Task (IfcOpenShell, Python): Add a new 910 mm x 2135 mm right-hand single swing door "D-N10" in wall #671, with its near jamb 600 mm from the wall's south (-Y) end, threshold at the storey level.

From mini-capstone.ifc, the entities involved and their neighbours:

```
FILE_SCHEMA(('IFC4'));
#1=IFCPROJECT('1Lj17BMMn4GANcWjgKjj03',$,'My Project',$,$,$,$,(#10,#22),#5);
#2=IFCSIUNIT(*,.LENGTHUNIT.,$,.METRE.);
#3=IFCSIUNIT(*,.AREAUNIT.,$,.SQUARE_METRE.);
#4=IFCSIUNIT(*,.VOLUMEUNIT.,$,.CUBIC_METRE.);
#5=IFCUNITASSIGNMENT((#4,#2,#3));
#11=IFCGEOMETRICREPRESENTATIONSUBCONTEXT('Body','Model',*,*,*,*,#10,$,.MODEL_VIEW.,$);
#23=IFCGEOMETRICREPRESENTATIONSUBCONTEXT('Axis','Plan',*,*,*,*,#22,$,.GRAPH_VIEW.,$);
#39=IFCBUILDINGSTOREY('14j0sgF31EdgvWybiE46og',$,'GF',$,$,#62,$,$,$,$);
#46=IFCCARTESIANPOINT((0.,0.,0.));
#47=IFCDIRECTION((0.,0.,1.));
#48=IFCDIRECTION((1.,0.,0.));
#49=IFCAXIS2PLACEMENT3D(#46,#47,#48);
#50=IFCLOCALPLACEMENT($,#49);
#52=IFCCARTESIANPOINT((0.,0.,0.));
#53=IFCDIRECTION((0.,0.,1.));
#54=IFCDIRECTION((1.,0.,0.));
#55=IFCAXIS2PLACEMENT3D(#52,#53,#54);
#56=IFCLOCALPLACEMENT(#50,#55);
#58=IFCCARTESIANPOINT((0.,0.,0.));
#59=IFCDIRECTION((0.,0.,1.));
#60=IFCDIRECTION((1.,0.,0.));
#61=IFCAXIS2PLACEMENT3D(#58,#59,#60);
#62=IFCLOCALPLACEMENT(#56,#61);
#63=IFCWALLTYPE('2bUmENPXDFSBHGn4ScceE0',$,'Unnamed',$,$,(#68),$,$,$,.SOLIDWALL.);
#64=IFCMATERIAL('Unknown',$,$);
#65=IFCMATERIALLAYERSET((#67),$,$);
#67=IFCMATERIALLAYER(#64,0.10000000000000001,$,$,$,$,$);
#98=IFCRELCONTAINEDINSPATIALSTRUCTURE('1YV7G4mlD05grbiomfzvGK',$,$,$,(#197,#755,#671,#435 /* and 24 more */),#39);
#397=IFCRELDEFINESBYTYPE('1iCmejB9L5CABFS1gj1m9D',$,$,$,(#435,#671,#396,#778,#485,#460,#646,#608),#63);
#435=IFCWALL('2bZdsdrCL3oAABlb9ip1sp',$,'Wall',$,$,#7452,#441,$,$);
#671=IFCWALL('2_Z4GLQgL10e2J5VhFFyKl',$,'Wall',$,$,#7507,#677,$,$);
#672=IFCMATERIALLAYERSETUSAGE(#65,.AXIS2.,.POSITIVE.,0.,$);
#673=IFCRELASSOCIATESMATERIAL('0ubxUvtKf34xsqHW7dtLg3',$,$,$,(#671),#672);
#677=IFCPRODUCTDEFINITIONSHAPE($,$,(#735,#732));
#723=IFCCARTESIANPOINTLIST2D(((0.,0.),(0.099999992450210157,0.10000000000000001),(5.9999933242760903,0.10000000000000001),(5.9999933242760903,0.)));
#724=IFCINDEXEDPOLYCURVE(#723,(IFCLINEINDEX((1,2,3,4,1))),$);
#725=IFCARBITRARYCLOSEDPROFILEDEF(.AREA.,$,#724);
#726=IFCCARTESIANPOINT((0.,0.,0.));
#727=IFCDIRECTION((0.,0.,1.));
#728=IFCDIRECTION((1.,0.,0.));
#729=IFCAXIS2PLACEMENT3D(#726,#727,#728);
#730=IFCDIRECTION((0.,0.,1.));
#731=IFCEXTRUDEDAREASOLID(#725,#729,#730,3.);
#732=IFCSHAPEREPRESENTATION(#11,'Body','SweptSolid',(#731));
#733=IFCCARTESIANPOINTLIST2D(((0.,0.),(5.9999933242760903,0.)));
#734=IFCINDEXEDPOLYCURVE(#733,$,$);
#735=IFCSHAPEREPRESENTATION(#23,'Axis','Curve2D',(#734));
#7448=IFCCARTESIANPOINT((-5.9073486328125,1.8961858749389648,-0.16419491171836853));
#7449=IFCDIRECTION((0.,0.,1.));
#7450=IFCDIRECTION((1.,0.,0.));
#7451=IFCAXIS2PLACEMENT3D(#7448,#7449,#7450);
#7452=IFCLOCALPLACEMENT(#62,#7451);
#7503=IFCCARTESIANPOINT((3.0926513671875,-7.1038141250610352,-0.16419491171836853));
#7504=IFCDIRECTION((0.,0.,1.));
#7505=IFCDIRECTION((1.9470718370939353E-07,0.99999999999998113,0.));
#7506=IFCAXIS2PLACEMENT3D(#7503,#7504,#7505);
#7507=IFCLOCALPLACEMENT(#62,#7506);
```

```python
import numpy as np
import ifcopenshell
import ifcopenshell.api.feature
import ifcopenshell.api.geometry
import ifcopenshell.api.root
import ifcopenshell.api.spatial
import ifcopenshell.geom
import ifcopenshell.util.element
import ifcopenshell.util.placement
import ifcopenshell.util.representation
import ifcopenshell.util.shape
import ifcopenshell.util.unit

model = ifcopenshell.open("mini-capstone.ifc")
unit_scale = ifcopenshell.util.unit.calculate_unit_scale(model)
settings = ifcopenshell.geom.settings()


def volume(element):
    """Net volume in cubic metres, openings subtracted."""
    shape = ifcopenshell.geom.create_shape(settings, element)
    return ifcopenshell.util.shape.get_volume(shape.geometry)


wall = model.by_guid("2_Z4GLQgL10e2J5VhFFyKl")
storey = ifcopenshell.util.element.get_container(wall, ifc_class="IfcBuildingStorey")
context = ifcopenshell.util.representation.get_context(model, "Model", "Body", "MODEL_VIEW")
before = volume(wall)

width, height, from_end, sill = 0.91, 2.135, 0.6, 0.0  # metres

# The wall runs along its own X axis, and the end named is its -X end.
wall_shape = ifcopenshell.geom.create_shape(settings, wall)
x, y, z = ifcopenshell.util.shape.get_vertices(wall_shape.geometry).T
start = x.min() + from_end
face, thickness = float(y.min()), float(y.max() - y.min())
wall_matrix = ifcopenshell.util.placement.get_local_placement(wall.ObjectPlacement)
level = ifcopenshell.util.placement.get_local_placement(storey.ObjectPlacement)[2, 3]


def in_wall(x, y):
    """Placement at x, y metres in the wall's axes, at sill height."""
    matrix = wall_matrix.copy()
    matrix[:, 3] = wall_matrix @ np.array([x / unit_scale, y / unit_scale, 0.0, 1.0])
    matrix[2, 3] = level + sill / unit_scale
    return matrix


# Opening: a box that overshoots both wall faces by 50 mm.
opening = ifcopenshell.api.root.create_entity(model, ifc_class="IfcOpeningElement", predefined_type="OPENING")
box = ifcopenshell.api.geometry.add_wall_representation(
    model, context=context, length=width, height=height, thickness=thickness + 0.1
)
ifcopenshell.api.geometry.assign_representation(model, product=opening, representation=box)
ifcopenshell.api.geometry.edit_object_placement(model, product=opening, matrix=in_wall(start, face - 0.05), is_si=False)
ifcopenshell.api.feature.add_feature(model, feature=opening, element=wall)

door = ifcopenshell.api.root.create_entity(model, ifc_class="IfcDoor", name="D-N10", predefined_type="DOOR")
door.OverallWidth, door.OverallHeight = width / unit_scale, height / unit_scale
door.OperationType = "SINGLE_SWING_RIGHT"
body = ifcopenshell.api.geometry.add_door_representation(
    model,
    context=context,
    overall_width=door.OverallWidth,
    overall_height=door.OverallHeight,
    operation_type="SINGLE_SWING_RIGHT",
    lining_properties={"LiningDepth": thickness / unit_scale, "ThresholdDepth": thickness / unit_scale},
)
ifcopenshell.api.geometry.assign_representation(model, product=door, representation=body)
ifcopenshell.api.spatial.assign_container(model, products=[door], relating_structure=storey)
ifcopenshell.api.feature.add_filling(model, opening=opening, element=door)

# The lining spans the wall, so the door starts at the wall face.
ifcopenshell.api.geometry.edit_object_placement(model, product=door, matrix=in_wall(start, face), is_si=False)

after = volume(wall)

print(f"wall volume {before:.3f} -> {after:.3f} m3")

model.write("mini-capstone_updated.ifc")
```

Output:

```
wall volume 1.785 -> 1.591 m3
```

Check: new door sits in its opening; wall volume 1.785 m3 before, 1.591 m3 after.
